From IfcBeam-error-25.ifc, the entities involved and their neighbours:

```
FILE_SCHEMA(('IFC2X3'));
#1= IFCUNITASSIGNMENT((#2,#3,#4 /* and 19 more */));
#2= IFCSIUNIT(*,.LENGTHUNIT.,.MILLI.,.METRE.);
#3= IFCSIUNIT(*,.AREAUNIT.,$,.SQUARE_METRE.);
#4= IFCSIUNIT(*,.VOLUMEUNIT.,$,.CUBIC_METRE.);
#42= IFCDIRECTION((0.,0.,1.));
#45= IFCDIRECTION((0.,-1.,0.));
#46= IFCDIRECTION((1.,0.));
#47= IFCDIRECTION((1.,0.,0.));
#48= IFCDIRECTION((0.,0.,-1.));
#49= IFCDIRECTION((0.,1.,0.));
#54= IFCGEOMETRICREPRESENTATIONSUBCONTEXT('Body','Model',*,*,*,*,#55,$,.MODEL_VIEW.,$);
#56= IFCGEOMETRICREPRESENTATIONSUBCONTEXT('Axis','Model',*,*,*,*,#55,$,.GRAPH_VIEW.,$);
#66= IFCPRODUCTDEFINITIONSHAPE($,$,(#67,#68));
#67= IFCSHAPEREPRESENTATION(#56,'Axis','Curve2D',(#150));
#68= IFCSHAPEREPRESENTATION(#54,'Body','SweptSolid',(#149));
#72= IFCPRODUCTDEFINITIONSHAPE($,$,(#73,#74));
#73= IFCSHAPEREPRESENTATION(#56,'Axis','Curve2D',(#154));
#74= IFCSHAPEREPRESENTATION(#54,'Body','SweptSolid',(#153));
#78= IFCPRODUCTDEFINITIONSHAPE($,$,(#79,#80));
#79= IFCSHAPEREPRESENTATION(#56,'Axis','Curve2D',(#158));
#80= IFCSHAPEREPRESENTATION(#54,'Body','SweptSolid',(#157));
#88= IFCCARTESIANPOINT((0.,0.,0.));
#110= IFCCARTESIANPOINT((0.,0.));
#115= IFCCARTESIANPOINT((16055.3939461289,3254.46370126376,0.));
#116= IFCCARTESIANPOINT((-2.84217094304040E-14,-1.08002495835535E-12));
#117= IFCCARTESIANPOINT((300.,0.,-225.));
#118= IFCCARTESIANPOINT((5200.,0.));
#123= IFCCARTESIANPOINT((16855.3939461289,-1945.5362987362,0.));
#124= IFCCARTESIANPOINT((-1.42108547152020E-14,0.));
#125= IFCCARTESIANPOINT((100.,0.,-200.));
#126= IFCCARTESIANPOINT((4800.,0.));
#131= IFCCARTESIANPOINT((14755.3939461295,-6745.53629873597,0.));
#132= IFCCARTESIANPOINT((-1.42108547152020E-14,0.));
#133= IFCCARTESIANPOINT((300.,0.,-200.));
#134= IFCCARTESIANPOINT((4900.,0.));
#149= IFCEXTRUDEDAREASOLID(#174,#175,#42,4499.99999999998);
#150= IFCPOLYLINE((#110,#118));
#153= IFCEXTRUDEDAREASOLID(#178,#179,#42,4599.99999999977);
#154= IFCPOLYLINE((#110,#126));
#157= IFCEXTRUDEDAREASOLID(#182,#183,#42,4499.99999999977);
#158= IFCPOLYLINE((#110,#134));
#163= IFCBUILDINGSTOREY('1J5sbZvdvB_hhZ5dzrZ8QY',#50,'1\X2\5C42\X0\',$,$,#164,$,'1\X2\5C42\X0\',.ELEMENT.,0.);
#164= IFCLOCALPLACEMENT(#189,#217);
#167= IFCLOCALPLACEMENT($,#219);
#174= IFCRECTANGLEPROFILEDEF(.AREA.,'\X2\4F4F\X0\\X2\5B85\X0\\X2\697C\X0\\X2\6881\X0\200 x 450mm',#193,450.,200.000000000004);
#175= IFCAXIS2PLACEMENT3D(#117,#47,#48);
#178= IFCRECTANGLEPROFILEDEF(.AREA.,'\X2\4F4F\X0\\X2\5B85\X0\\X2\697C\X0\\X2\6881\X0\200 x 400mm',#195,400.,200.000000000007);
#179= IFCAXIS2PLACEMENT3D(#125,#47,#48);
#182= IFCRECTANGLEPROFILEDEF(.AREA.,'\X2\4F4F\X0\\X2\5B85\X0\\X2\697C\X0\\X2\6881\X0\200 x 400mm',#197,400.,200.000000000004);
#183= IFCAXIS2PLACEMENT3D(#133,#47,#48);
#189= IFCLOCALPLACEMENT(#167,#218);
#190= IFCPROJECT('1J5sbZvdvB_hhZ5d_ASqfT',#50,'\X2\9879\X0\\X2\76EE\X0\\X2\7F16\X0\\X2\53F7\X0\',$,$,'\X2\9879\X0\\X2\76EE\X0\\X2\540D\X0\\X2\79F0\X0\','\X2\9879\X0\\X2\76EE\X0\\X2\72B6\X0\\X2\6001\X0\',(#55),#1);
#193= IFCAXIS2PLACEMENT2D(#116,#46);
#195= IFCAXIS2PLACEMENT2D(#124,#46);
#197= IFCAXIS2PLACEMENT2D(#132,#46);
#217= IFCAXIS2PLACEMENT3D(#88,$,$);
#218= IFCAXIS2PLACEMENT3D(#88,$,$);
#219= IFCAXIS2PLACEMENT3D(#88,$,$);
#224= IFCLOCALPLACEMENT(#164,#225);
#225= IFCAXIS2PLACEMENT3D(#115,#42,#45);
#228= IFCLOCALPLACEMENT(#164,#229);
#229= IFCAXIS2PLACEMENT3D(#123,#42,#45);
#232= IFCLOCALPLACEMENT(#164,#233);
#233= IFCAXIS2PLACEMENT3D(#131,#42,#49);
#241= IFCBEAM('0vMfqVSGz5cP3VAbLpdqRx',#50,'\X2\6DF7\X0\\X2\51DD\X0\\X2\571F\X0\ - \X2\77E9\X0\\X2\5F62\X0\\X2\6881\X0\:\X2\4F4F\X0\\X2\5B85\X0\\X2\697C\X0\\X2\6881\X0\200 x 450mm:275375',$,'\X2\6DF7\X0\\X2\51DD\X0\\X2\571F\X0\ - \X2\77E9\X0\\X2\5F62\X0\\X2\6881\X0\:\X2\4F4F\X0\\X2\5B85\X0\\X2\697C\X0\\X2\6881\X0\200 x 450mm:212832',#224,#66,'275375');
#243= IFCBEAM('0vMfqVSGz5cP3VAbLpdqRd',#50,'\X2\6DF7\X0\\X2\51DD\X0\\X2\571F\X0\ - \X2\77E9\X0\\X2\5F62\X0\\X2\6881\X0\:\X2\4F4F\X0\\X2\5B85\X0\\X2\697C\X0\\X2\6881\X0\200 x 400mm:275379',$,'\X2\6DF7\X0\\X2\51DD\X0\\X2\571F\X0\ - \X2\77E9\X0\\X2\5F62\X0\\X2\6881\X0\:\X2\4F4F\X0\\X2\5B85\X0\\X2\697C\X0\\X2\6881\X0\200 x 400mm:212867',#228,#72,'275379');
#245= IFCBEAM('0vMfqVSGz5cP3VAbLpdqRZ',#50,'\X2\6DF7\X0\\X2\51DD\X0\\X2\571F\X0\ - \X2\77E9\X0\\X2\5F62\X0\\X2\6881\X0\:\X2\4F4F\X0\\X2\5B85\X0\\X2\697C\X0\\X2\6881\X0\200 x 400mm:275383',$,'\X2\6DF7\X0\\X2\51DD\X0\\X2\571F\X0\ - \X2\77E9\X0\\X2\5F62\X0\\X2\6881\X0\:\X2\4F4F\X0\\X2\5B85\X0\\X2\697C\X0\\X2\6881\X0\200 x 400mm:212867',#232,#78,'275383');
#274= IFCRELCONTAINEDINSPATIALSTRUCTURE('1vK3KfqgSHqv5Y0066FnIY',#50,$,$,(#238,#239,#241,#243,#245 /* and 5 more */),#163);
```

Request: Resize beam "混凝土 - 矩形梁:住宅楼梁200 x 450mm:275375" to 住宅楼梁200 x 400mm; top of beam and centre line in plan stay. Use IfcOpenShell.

```python
import ifcopenshell
import ifcopenshell.util.element
import ifcopenshell.util.representation

model = ifcopenshell.open("IfcBeam-error-25.ifc")

member = model.by_guid("0vMfqVSGz5cP3VAbLpdqRx")
source = next(p for p in model.by_type("IfcRectangleProfileDef") if p.ProfileName == "住宅楼梁200 x 400mm")

body = ifcopenshell.util.representation.get_representation(member, "Model", "Body")
solid = body.Items[0]
old_profile = solid.SweptArea

# Copy the section's sizes but keep this member's own profile position.
profile = ifcopenshell.util.element.copy(model, source)
# Profiles are centred, so shift by half the change in depth to hold the top.
shift = (old_profile.XDim - profile.XDim) / 2
x, y = old_profile.Position.Location.Coordinates
up = (-1.0, 0.0)  # upwards, in the solid's own plane
location = model.createIfcCartesianPoint((x + up[0] * shift, y + up[1] * shift))
profile.Position = model.createIfcAxis2Placement2D(location, old_profile.Position.RefDirection)
solid.SweptArea = profile
if not model.get_total_inverses(old_profile):
    ifcopenshell.util.element.remove_deep2(model, old_profile)
member.Name = member.Name.replace("住宅楼梁200 x 450mm", "住宅楼梁200 x 400mm")
member.ObjectType = member.ObjectType.replace("住宅楼梁200 x 450mm", "住宅楼梁200 x 400mm")

print(solid.SweptArea)

model.write("IfcBeam-error-25_v2.ifc")
```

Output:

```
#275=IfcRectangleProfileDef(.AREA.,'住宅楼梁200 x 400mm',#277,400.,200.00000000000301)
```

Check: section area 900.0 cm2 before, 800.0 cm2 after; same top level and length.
